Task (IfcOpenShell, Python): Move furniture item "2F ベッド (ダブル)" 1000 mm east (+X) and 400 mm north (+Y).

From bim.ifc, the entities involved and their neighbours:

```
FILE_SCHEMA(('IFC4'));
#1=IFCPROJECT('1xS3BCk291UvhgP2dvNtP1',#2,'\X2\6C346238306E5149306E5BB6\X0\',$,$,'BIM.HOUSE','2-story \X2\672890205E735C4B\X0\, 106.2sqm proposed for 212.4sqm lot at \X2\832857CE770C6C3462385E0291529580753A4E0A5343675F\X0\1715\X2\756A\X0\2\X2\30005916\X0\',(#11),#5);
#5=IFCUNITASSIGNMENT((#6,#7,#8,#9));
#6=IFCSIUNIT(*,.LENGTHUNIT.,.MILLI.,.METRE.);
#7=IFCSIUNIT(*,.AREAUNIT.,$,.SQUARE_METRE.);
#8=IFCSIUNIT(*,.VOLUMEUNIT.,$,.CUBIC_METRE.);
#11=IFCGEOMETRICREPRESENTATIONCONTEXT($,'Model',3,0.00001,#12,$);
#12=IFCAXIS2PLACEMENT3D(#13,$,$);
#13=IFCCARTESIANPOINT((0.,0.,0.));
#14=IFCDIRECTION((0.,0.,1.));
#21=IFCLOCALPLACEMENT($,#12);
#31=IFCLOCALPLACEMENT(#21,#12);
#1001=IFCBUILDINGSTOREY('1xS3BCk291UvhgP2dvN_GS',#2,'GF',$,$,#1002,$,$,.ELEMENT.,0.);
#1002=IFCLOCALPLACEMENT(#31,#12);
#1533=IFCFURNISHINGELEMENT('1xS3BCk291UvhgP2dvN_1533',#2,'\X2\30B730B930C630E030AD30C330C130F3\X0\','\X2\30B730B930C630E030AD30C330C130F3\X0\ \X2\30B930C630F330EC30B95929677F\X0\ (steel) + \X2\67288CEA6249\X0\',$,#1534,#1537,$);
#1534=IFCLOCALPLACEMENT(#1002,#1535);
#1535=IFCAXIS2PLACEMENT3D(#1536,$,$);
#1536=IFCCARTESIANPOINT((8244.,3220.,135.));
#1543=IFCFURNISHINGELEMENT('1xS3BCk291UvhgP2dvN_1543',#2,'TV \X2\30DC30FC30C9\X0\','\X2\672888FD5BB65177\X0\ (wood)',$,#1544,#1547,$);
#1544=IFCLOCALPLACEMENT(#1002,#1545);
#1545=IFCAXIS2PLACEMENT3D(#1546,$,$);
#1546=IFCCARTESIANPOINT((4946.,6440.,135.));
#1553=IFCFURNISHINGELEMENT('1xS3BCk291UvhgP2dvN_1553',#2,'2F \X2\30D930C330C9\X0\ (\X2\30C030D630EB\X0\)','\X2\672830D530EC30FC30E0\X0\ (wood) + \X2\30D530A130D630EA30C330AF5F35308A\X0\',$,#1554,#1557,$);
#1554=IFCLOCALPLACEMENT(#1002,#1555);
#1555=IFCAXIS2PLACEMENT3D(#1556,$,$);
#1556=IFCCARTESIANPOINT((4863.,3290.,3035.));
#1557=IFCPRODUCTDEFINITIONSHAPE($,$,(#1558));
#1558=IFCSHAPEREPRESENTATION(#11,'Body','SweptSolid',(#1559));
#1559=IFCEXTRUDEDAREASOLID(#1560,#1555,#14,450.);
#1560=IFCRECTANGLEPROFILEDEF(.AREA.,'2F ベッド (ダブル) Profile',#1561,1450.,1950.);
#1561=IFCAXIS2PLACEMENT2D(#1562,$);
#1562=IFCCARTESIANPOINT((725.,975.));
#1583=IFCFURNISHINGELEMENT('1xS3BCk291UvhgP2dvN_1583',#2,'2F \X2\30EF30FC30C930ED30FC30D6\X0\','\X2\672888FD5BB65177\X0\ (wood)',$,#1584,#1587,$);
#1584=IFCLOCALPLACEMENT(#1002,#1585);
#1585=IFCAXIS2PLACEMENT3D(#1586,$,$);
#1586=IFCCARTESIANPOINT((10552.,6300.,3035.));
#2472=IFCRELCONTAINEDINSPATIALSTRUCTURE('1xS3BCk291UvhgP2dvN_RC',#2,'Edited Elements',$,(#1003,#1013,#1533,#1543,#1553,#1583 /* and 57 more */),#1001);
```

```python
import ifcopenshell
import ifcopenshell.api.geometry
import ifcopenshell.util.placement
import ifcopenshell.util.unit

model = ifcopenshell.open("bim.ifc")
unit_scale = ifcopenshell.util.unit.calculate_unit_scale(model)

item = model.by_id(1553)
matrix = ifcopenshell.util.placement.get_local_placement(item.ObjectPlacement)
matrix[0, 3] += 1 / unit_scale
matrix[1, 3] += 0.4 / unit_scale
ifcopenshell.api.geometry.edit_object_placement(model, product=item, matrix=matrix, is_si=False)

print(ifcopenshell.util.placement.get_local_placement(item.ObjectPlacement).round(3) + 0.0)

model.write("bim_v2.ifc")
```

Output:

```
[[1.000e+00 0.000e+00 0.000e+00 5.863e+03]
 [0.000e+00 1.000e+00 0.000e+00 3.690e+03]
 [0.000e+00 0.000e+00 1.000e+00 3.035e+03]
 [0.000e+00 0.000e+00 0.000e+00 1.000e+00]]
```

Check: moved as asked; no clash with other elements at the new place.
